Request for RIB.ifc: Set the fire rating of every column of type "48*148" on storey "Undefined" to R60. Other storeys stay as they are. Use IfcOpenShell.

First a look at what the model holds.

```python
import ifcopenshell
import ifcopenshell.util.element

model = ifcopenshell.open("RIB.ifc")
print(model.schema)
storey = next(s for s in model.by_type("IfcBuildingStorey") if s.Name == "Undefined")
columns = [e for e in ifcopenshell.util.element.get_decomposition(storey) if e.is_a("IfcColumn")]
seen = {}
for e in columns:
    element_type = ifcopenshell.util.element.get_type(e)
    key = (element_type.Name if element_type != e and element_type else None, ifcopenshell.util.element.get_pset(e, "Pset_ColumnCommon", "FireRating"))
    seen[key] = seen.get(key, 0) + 1
for (name, value), count in sorted(seen.items(), key=str):
    print(count, "x", name, "|", value)
```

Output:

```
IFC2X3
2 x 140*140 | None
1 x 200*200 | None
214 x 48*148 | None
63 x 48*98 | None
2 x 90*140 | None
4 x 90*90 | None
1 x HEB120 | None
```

```python
import ifcopenshell
import ifcopenshell.api.pset
import ifcopenshell.util.element

model = ifcopenshell.open("RIB.ifc")

storey = next(s for s in model.by_type("IfcBuildingStorey") if s.Name == "Undefined")
columns = [e for e in ifcopenshell.util.element.get_decomposition(storey) if e.is_a("IfcColumn")]

count = 0
for e in columns:
    element_type = ifcopenshell.util.element.get_type(e)
    if element_type in (None, e) or element_type.Name != "48*148":
        continue
    # add_pset returns the element's existing set when there is one.
    pset = ifcopenshell.api.pset.add_pset(model, product=e, name="Pset_ColumnCommon")
    ifcopenshell.api.pset.edit_pset(model, pset=pset, properties={"FireRating": "R60"})
    count += 1

print(count, "columns updated")

model.write("RIB-out.ifc")
```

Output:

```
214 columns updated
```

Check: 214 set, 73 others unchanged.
